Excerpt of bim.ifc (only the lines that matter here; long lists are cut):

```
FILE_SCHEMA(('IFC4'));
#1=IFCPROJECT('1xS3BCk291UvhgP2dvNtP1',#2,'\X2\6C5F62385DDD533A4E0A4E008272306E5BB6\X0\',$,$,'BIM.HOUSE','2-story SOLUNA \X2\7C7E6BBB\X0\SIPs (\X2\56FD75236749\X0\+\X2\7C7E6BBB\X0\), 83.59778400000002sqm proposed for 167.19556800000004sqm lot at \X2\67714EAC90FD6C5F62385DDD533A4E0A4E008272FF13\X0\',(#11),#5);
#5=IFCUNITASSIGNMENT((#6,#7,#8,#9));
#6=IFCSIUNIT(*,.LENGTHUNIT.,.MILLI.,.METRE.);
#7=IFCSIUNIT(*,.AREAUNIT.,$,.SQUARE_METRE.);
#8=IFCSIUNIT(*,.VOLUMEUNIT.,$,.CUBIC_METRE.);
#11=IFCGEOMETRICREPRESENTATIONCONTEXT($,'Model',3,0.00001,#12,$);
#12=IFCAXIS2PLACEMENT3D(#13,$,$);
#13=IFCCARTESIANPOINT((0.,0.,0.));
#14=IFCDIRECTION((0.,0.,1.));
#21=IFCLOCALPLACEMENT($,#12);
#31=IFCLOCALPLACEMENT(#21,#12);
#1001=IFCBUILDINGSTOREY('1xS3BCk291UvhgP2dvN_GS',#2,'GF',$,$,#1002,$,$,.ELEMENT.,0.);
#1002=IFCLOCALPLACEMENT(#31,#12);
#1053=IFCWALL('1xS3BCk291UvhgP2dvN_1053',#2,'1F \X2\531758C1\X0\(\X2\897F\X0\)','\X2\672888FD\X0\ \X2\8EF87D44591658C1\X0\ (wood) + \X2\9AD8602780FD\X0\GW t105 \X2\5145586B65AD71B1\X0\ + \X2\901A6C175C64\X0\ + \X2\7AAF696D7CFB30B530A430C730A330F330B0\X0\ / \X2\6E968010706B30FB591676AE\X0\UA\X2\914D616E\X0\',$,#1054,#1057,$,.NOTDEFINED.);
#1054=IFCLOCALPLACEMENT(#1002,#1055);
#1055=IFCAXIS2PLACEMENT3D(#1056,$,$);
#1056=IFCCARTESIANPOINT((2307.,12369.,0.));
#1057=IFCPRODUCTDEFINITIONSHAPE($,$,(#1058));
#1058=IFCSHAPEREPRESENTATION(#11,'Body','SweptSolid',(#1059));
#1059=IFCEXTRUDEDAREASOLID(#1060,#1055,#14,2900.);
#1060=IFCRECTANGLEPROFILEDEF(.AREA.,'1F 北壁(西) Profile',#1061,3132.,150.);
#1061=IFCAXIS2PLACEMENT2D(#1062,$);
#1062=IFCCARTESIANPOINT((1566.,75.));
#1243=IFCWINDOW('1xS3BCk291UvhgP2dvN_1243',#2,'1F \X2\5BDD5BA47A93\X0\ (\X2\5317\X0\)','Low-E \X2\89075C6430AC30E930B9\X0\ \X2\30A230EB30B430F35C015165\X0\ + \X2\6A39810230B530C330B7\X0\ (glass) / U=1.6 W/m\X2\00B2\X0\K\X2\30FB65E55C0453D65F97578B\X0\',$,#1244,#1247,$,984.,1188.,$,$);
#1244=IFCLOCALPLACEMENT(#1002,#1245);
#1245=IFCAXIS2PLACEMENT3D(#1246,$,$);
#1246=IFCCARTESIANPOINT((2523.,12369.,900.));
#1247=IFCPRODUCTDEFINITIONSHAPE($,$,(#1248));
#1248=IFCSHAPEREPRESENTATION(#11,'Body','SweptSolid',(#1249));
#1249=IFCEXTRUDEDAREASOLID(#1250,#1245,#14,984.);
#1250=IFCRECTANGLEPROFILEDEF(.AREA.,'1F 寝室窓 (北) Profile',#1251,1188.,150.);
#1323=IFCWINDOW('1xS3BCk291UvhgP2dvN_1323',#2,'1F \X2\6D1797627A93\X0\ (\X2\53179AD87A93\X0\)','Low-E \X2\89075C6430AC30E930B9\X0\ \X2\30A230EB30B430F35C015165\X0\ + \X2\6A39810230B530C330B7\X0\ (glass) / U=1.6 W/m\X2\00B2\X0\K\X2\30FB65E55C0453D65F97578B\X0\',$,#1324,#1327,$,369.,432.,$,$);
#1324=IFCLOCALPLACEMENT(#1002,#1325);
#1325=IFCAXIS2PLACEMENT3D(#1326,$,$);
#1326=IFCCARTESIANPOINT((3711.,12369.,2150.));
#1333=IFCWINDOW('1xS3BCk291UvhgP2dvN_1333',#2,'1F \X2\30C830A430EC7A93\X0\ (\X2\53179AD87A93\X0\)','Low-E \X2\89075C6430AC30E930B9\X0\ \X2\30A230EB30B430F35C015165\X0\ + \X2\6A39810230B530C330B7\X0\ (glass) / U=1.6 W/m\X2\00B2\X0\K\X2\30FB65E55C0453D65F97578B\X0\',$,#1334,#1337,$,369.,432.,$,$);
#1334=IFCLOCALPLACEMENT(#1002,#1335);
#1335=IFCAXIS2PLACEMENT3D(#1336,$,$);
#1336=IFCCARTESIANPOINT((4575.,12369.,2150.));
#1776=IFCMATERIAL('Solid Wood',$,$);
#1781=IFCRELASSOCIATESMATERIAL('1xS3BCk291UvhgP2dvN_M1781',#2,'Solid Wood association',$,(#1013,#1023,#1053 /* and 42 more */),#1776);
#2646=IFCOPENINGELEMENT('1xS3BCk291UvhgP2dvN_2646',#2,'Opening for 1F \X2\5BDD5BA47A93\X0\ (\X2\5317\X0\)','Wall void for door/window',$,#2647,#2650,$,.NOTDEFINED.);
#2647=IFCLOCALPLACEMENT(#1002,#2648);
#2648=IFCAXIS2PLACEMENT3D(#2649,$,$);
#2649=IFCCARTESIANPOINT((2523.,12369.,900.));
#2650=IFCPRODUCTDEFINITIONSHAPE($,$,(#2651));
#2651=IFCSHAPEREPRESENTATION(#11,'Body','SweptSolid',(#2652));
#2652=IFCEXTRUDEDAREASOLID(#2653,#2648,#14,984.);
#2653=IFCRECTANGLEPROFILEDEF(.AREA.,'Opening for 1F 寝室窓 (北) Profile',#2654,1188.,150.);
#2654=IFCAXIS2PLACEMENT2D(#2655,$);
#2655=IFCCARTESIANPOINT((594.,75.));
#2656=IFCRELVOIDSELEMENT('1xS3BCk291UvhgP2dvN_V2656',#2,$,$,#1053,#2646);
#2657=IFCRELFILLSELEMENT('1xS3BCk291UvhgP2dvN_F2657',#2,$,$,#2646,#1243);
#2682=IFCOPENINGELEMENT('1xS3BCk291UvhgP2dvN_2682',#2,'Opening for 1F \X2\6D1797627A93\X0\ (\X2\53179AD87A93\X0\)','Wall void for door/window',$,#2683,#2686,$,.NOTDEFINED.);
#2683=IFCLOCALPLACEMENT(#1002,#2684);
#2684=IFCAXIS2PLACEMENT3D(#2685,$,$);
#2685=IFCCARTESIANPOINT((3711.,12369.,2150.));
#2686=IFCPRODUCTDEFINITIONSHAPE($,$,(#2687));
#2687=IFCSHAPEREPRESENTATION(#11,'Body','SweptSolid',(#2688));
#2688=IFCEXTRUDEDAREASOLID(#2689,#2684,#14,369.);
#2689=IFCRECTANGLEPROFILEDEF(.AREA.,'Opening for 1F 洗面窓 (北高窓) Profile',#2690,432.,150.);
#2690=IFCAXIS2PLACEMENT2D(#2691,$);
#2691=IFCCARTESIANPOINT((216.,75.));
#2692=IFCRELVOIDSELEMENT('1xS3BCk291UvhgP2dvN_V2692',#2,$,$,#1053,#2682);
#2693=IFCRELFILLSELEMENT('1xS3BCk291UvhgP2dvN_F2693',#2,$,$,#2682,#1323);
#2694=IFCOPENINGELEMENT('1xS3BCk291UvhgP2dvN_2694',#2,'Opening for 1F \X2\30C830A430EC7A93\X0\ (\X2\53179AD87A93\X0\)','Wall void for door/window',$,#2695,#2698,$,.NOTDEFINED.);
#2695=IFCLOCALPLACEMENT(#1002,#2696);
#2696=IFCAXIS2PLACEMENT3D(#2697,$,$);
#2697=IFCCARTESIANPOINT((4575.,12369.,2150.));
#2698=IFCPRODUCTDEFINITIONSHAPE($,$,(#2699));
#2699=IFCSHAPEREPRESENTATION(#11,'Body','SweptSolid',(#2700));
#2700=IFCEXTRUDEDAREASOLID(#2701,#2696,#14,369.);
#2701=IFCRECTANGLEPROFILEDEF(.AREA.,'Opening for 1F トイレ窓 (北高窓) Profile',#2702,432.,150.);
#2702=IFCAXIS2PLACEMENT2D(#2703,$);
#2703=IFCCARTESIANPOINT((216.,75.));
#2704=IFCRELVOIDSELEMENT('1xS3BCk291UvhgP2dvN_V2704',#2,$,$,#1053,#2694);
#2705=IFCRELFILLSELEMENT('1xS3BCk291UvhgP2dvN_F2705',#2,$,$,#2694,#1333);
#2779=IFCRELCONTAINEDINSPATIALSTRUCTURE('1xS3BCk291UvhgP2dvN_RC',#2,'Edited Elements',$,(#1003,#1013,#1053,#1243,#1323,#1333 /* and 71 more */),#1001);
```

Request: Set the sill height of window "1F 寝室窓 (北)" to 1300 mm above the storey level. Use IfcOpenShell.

```python
import numpy as np
import ifcopenshell
import ifcopenshell.api.geometry
import ifcopenshell.geom
import ifcopenshell.util.element
import ifcopenshell.util.placement
import ifcopenshell.util.shape
import ifcopenshell.util.unit

model = ifcopenshell.open("bim.ifc")
unit_scale = ifcopenshell.util.unit.calculate_unit_scale(model)

window = model.by_guid("1xS3BCk291UvhgP2dvN_1243")
opening = window.FillsVoids[0].RelatingOpeningElement
storey = ifcopenshell.util.element.get_container(window, ifc_class="IfcBuildingStorey")
level = ifcopenshell.util.placement.get_local_placement(storey.ObjectPlacement)[2, 3]

# The opening's origin need not be at the sill, so measure its lowest point.
shape = ifcopenshell.geom.create_shape(ifcopenshell.geom.settings(), opening)
bottom = ifcopenshell.util.shape.get_shape_bottom_elevation(shape, shape.geometry) / unit_scale
dz = level + 1300.0 - bottom

shift = np.array([0.0, 0.0, dz])
# The window is not placed relative to its opening, so move both.
for product in (opening, window):
    matrix = ifcopenshell.util.placement.get_local_placement(product.ObjectPlacement)
    matrix[:3, 3] += shift
    ifcopenshell.api.geometry.edit_object_placement(model, product=product, matrix=matrix, is_si=False)

print(f"moved by {dz * unit_scale:+.3f} m")

model.write("bim_rev.ifc")
```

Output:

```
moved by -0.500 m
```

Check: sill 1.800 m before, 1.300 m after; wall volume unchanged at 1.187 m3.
